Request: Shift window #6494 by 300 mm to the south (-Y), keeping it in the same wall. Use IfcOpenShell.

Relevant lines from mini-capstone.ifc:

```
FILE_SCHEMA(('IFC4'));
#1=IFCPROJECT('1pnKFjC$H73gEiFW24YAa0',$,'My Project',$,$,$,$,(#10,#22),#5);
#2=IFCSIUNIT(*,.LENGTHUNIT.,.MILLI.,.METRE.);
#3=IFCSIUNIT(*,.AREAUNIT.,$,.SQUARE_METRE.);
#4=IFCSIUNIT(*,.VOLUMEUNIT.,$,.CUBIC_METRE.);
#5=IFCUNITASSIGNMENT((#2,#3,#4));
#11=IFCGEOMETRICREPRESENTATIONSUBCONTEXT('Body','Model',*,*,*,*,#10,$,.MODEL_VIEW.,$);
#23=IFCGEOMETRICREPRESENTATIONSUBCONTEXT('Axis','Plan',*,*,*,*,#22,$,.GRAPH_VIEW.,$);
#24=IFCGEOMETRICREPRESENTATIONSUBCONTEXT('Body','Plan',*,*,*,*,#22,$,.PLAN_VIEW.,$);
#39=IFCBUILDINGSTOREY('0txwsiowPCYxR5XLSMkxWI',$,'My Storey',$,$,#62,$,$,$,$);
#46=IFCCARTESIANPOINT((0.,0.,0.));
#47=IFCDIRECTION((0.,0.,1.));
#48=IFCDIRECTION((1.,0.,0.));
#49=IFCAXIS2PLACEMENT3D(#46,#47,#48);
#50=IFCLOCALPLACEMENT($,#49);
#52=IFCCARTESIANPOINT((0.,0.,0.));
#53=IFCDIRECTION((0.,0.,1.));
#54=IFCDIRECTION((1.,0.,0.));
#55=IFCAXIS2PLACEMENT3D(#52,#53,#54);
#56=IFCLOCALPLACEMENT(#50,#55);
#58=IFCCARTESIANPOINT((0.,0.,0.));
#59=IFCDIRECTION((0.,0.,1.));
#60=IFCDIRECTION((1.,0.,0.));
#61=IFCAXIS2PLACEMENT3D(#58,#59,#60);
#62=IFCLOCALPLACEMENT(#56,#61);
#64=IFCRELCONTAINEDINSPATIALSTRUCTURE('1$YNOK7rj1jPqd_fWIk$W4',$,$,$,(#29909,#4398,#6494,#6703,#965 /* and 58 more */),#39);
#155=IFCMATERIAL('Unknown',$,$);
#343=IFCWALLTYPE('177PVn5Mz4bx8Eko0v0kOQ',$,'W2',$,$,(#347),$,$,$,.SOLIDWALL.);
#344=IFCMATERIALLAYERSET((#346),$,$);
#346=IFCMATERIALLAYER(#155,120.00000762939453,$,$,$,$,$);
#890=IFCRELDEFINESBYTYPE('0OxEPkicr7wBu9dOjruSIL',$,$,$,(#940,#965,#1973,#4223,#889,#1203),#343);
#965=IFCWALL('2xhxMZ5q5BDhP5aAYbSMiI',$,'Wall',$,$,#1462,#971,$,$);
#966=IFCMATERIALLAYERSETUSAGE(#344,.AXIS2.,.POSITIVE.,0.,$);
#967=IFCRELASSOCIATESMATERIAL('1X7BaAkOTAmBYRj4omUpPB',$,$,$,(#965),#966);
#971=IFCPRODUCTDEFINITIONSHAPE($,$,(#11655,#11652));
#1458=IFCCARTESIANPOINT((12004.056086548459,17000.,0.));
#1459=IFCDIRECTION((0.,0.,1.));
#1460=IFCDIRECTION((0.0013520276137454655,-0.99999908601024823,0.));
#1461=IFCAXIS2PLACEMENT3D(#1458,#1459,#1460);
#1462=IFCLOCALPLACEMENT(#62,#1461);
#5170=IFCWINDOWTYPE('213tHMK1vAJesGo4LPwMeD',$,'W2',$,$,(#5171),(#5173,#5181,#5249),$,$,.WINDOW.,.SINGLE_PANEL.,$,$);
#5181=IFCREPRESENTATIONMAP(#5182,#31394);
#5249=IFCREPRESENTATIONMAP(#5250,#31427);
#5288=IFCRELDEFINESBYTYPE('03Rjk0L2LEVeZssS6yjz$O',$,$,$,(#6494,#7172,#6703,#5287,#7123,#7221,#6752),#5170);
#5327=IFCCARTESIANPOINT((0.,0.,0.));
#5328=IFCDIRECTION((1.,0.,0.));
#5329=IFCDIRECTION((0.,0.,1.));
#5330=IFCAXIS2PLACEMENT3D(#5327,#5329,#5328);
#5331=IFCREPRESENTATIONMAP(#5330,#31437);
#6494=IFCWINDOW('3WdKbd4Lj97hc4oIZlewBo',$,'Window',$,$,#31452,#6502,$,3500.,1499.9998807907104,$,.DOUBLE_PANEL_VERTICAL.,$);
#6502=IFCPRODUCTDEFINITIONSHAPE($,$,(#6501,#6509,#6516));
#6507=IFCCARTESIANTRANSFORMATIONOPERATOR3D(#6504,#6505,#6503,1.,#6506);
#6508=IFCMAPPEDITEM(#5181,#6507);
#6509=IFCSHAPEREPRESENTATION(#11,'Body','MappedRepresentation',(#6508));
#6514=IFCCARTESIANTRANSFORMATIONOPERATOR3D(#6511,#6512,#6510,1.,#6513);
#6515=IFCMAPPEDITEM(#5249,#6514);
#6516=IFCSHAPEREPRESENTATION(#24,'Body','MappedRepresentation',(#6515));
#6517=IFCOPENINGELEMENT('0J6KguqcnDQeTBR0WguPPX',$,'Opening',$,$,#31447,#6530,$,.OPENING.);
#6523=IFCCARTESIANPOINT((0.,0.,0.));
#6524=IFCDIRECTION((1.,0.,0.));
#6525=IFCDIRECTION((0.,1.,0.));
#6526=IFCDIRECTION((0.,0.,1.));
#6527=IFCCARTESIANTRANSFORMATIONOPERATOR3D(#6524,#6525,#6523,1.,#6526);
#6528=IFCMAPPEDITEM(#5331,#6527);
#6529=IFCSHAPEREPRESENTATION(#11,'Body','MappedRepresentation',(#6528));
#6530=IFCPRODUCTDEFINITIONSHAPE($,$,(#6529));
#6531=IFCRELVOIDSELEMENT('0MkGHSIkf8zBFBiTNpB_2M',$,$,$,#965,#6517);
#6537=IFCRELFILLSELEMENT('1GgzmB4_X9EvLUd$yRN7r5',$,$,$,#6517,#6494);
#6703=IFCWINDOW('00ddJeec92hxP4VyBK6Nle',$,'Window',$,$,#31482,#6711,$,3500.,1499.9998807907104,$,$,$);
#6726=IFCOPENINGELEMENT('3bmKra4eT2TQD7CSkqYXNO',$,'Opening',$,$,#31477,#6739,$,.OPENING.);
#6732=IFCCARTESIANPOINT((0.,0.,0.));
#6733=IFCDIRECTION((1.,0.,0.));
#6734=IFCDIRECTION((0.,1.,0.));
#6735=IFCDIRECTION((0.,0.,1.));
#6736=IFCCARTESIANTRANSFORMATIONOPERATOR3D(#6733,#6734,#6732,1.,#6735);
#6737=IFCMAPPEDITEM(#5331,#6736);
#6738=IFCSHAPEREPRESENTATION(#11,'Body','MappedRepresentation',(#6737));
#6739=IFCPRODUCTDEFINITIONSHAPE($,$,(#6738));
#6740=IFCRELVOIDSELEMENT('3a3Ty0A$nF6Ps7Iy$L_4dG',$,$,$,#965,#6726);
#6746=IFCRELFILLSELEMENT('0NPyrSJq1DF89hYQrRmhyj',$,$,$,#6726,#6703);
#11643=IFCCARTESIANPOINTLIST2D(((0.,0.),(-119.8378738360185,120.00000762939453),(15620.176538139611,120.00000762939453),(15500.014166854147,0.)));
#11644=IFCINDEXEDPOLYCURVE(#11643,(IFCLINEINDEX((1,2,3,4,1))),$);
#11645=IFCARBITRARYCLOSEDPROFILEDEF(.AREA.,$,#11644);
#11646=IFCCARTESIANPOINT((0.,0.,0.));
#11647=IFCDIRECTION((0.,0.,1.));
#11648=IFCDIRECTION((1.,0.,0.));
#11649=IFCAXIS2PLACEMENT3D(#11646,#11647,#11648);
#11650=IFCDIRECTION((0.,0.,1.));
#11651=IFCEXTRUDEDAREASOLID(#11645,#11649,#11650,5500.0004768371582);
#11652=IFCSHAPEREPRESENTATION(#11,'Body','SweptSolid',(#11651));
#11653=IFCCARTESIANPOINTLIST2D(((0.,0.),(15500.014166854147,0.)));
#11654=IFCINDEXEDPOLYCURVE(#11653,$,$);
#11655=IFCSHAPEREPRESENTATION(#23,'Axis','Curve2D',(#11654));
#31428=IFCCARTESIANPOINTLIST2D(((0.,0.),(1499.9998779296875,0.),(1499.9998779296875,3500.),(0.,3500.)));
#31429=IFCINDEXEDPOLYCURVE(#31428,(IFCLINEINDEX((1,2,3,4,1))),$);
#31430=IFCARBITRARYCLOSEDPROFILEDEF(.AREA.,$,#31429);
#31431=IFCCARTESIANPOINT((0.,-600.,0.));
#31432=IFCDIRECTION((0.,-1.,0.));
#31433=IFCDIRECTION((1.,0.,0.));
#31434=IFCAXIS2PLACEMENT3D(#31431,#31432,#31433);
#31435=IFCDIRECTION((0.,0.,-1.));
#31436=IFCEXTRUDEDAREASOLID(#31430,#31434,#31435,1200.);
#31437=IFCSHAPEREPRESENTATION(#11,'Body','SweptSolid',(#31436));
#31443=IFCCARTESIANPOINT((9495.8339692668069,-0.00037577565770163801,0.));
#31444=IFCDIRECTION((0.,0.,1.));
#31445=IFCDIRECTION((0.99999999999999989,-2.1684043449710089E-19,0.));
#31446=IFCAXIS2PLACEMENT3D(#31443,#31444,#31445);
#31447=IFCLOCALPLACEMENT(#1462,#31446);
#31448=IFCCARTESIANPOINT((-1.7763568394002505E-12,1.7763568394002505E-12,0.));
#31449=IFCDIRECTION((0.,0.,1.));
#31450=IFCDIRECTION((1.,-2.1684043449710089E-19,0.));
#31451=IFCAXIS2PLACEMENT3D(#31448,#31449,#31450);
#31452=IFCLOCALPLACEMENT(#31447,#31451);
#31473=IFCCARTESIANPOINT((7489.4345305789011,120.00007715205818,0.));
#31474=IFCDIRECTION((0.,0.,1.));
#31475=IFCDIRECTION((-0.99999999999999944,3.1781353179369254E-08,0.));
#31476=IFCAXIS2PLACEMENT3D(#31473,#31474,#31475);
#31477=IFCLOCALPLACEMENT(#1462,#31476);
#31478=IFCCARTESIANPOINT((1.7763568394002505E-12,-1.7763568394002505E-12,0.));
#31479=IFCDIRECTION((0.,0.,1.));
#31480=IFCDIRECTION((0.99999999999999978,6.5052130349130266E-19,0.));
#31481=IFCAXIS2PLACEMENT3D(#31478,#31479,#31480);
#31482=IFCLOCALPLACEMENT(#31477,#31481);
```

```python
import ifcopenshell
import ifcopenshell.api.geometry
import ifcopenshell.util.placement
import ifcopenshell.util.unit

model = ifcopenshell.open("mini-capstone.ifc")
unit_scale = ifcopenshell.util.unit.calculate_unit_scale(model)

window = model.by_id(6494)
opening = window.FillsVoids[0].RelatingOpeningElement
wall = opening.VoidsElements[0].RelatingBuildingElement

wall_matrix = ifcopenshell.util.placement.get_local_placement(wall.ObjectPlacement)
shift = wall_matrix[:3, 0] * 0.3 / unit_scale
before = ifcopenshell.util.placement.get_local_placement(window.ObjectPlacement)[:3, 3].copy()

# The window is placed relative to its opening, so it follows when the opening moves.
matrix = ifcopenshell.util.placement.get_local_placement(opening.ObjectPlacement)
matrix[:3, 3] += shift
ifcopenshell.api.geometry.edit_object_placement(
    model, product=opening, matrix=matrix, is_si=False, should_transform_children=True
)

after = ifcopenshell.util.placement.get_local_placement(window.ObjectPlacement)[:3, 3]
print("window moved by", (after - before).round(3) + 0.0)

model.write("mini-capstone_rev.ifc")
```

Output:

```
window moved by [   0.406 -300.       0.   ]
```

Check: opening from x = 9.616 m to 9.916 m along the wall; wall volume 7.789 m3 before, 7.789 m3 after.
